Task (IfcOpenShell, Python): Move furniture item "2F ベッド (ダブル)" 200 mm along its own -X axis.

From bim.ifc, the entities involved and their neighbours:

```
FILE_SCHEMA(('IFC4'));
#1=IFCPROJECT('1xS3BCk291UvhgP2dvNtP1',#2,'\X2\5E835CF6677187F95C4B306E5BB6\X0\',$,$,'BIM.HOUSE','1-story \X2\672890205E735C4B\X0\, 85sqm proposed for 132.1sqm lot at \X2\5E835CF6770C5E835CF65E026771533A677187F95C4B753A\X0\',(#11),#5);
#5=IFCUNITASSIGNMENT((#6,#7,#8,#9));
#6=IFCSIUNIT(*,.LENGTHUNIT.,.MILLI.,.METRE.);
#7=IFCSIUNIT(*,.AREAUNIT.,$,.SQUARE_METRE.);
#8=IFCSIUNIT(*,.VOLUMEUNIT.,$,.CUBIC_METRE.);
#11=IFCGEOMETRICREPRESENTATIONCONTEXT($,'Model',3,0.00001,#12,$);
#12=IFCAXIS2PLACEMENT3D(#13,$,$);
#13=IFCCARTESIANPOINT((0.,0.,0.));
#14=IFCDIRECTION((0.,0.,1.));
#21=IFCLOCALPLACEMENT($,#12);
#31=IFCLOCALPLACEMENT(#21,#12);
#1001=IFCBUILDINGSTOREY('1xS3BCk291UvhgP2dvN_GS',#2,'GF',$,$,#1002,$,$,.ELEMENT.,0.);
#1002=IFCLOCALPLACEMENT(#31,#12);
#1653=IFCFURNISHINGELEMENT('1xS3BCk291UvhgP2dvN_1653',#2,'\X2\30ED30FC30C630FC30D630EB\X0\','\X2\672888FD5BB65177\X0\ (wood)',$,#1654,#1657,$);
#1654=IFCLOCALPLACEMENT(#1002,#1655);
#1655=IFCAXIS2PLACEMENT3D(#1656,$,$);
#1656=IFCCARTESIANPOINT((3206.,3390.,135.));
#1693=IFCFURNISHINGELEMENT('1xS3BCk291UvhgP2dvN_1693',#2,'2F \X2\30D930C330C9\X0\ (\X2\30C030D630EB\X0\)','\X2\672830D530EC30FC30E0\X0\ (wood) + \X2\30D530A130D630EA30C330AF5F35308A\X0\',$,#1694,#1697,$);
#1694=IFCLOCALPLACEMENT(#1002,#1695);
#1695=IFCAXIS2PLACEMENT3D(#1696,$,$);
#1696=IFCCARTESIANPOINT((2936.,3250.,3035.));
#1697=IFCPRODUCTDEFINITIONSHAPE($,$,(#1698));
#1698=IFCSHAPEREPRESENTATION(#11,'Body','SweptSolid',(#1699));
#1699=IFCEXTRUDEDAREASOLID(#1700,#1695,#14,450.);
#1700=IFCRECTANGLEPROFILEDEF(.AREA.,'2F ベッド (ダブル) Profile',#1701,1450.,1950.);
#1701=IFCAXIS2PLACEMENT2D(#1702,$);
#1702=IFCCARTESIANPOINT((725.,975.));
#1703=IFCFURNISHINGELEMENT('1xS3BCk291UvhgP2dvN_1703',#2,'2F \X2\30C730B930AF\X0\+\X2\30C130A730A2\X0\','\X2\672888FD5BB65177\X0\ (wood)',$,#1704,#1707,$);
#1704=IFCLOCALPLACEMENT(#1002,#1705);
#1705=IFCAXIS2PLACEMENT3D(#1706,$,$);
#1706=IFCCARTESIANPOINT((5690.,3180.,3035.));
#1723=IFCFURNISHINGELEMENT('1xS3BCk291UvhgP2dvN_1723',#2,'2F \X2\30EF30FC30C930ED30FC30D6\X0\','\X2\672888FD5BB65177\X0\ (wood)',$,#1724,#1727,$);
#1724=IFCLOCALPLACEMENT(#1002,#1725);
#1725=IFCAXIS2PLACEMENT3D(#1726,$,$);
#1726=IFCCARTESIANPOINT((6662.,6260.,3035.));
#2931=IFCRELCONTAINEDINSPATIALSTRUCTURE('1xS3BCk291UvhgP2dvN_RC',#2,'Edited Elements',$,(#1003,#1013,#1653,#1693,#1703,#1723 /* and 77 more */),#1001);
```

```python
import ifcopenshell
import ifcopenshell.api.geometry
import ifcopenshell.util.placement

model = ifcopenshell.open("bim.ifc")

item = model.by_guid("1xS3BCk291UvhgP2dvN_1693")
matrix = ifcopenshell.util.placement.get_local_placement(item.ObjectPlacement)
matrix[:3, 3] -= matrix[:3, 0] * 200.0
ifcopenshell.api.geometry.edit_object_placement(model, product=item, matrix=matrix, is_si=False)

print(ifcopenshell.util.placement.get_local_placement(item.ObjectPlacement).round(3) + 0.0)

model.write("bim_rev.ifc")
```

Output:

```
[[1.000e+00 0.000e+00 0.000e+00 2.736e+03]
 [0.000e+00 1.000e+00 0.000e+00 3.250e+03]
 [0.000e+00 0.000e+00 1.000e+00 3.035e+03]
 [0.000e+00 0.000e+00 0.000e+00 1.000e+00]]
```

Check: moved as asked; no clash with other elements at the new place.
